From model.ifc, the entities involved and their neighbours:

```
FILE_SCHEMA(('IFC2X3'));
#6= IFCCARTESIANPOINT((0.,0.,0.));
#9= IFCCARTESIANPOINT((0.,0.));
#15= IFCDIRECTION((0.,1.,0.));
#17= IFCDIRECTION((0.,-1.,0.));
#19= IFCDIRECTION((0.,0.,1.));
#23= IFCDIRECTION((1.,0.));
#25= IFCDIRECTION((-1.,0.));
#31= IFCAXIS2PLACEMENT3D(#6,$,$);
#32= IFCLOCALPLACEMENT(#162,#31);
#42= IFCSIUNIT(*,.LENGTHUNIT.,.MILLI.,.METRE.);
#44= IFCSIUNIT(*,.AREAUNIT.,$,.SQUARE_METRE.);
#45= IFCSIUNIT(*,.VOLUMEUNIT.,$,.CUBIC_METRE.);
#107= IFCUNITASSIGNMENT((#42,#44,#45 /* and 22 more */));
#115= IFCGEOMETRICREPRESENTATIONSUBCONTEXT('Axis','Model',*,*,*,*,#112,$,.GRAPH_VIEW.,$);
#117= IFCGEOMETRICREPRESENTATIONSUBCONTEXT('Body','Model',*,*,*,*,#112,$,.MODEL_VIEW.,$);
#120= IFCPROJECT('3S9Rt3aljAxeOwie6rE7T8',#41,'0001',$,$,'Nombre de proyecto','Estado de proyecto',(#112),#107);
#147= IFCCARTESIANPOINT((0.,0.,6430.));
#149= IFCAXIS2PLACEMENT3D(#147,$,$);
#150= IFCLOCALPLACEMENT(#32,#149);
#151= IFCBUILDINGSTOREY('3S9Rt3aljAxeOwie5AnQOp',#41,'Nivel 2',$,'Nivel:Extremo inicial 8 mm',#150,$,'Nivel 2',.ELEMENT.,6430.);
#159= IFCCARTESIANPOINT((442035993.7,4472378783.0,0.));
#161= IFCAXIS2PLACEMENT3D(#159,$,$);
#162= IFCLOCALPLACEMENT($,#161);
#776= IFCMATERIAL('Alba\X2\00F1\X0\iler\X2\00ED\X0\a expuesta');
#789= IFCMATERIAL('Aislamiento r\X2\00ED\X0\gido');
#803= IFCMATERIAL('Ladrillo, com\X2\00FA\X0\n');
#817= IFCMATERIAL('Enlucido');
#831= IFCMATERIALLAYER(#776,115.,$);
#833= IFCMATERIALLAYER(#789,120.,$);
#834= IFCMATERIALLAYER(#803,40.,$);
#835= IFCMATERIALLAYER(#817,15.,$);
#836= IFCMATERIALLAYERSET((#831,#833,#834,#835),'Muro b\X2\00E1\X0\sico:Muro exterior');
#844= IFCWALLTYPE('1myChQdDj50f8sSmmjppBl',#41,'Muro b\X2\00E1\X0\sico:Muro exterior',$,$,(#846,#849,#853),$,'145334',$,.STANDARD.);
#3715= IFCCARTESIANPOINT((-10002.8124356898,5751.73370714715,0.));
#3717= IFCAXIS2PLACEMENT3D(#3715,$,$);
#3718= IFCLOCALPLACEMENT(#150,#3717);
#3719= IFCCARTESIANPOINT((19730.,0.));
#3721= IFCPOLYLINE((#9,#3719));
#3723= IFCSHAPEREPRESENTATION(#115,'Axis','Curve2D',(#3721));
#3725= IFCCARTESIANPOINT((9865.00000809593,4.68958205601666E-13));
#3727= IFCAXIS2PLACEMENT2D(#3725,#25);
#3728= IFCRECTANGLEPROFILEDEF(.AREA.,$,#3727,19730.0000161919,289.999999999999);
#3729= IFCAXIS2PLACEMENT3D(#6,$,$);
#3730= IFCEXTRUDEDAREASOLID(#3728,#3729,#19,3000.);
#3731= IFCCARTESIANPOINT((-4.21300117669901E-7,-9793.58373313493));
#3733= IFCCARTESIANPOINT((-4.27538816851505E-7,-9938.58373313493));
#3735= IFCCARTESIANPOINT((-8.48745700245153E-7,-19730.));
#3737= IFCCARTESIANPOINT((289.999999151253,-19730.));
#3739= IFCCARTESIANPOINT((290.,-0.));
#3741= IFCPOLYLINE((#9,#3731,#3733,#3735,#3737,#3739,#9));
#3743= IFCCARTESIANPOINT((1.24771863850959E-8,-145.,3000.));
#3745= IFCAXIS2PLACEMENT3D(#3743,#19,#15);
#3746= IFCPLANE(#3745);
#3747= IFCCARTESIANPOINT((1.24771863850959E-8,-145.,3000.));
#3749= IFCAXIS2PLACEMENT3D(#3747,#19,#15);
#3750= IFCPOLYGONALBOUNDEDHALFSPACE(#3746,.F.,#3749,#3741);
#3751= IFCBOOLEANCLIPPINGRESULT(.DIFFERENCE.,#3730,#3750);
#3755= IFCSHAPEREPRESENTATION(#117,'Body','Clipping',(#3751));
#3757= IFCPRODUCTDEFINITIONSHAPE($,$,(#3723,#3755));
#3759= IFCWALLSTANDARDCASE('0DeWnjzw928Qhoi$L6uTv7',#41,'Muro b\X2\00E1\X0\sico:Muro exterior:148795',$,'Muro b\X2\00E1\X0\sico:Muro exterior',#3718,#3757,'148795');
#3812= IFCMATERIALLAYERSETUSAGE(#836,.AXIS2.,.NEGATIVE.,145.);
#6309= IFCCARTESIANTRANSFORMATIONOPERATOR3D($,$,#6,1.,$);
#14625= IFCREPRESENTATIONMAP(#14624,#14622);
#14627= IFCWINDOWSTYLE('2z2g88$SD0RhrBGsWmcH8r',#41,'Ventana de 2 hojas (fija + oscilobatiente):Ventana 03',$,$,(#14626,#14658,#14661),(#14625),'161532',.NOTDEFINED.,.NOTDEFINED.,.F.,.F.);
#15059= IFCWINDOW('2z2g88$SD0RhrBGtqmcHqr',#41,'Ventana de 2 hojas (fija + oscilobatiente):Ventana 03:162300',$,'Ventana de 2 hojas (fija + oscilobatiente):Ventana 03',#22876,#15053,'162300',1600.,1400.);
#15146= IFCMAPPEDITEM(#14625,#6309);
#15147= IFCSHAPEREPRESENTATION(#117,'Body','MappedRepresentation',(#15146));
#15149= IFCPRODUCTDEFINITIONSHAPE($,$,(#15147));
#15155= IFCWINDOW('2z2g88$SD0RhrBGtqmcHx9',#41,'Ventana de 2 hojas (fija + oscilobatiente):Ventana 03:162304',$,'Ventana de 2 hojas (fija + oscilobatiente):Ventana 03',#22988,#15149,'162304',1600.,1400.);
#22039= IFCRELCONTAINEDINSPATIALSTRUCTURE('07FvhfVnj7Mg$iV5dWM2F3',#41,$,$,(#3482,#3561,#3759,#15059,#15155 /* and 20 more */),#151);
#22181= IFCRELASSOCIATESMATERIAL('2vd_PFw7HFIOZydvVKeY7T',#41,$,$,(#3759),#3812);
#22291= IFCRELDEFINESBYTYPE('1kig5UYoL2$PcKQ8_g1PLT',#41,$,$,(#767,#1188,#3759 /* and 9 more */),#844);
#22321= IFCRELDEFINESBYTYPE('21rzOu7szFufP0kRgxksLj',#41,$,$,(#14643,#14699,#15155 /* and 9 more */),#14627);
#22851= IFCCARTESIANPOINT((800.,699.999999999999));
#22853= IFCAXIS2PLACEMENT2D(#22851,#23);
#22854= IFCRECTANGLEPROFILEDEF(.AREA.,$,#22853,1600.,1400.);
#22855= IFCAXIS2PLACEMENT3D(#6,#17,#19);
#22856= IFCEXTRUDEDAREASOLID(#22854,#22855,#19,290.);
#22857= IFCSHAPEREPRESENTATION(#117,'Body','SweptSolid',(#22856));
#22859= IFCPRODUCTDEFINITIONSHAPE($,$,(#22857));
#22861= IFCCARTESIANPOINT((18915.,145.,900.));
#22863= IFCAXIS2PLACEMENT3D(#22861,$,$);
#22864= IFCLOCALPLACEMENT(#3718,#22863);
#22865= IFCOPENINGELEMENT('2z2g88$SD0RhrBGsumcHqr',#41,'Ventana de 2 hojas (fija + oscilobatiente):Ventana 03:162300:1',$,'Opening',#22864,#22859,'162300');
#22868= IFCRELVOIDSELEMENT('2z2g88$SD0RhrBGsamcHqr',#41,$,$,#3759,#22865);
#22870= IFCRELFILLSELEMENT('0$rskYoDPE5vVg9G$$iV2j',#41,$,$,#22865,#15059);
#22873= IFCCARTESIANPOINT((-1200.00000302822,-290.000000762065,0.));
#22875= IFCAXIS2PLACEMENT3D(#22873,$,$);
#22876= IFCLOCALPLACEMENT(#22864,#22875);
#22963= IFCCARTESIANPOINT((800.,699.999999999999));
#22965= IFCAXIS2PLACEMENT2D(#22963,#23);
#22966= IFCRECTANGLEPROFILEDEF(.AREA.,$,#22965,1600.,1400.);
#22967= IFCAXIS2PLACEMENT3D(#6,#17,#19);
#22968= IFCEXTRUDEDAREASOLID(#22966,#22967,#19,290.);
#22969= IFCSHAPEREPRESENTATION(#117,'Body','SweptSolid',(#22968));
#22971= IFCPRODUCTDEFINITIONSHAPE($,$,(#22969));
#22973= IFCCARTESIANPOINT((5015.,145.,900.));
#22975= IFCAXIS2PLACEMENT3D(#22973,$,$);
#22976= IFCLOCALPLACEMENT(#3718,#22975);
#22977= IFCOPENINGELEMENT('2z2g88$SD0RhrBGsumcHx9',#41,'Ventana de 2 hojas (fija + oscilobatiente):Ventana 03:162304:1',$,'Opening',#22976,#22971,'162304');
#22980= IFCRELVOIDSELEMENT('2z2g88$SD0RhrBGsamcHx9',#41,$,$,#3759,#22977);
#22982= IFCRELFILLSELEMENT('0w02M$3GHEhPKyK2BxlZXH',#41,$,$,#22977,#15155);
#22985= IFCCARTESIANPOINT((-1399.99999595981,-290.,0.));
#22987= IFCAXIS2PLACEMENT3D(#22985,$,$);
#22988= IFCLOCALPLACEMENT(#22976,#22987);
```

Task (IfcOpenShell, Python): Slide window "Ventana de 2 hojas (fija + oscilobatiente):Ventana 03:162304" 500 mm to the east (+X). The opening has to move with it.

```python
import ifcopenshell
import ifcopenshell.api.geometry
import ifcopenshell.util.placement

model = ifcopenshell.open("model.ifc")

window = model.by_guid("2z2g88$SD0RhrBGtqmcHx9")
opening = window.FillsVoids[0].RelatingOpeningElement
wall = opening.VoidsElements[0].RelatingBuildingElement

wall_matrix = ifcopenshell.util.placement.get_local_placement(wall.ObjectPlacement)
shift = wall_matrix[:3, 0] * 500.0
before = ifcopenshell.util.placement.get_local_placement(window.ObjectPlacement)[:3, 3].copy()

# The window is placed relative to its opening, so it follows when the opening moves.
matrix = ifcopenshell.util.placement.get_local_placement(opening.ObjectPlacement)
matrix[:3, 3] += shift
ifcopenshell.api.geometry.edit_object_placement(
    model, product=opening, matrix=matrix, is_si=False, should_transform_children=True
)

after = ifcopenshell.util.placement.get_local_placement(window.ObjectPlacement)[:3, 3]
print("window moved by", (after - before).round(3) + 0.0)

model.write("model_v2.ifc")
```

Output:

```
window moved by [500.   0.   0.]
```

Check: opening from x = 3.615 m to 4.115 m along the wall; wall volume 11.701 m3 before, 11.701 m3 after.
